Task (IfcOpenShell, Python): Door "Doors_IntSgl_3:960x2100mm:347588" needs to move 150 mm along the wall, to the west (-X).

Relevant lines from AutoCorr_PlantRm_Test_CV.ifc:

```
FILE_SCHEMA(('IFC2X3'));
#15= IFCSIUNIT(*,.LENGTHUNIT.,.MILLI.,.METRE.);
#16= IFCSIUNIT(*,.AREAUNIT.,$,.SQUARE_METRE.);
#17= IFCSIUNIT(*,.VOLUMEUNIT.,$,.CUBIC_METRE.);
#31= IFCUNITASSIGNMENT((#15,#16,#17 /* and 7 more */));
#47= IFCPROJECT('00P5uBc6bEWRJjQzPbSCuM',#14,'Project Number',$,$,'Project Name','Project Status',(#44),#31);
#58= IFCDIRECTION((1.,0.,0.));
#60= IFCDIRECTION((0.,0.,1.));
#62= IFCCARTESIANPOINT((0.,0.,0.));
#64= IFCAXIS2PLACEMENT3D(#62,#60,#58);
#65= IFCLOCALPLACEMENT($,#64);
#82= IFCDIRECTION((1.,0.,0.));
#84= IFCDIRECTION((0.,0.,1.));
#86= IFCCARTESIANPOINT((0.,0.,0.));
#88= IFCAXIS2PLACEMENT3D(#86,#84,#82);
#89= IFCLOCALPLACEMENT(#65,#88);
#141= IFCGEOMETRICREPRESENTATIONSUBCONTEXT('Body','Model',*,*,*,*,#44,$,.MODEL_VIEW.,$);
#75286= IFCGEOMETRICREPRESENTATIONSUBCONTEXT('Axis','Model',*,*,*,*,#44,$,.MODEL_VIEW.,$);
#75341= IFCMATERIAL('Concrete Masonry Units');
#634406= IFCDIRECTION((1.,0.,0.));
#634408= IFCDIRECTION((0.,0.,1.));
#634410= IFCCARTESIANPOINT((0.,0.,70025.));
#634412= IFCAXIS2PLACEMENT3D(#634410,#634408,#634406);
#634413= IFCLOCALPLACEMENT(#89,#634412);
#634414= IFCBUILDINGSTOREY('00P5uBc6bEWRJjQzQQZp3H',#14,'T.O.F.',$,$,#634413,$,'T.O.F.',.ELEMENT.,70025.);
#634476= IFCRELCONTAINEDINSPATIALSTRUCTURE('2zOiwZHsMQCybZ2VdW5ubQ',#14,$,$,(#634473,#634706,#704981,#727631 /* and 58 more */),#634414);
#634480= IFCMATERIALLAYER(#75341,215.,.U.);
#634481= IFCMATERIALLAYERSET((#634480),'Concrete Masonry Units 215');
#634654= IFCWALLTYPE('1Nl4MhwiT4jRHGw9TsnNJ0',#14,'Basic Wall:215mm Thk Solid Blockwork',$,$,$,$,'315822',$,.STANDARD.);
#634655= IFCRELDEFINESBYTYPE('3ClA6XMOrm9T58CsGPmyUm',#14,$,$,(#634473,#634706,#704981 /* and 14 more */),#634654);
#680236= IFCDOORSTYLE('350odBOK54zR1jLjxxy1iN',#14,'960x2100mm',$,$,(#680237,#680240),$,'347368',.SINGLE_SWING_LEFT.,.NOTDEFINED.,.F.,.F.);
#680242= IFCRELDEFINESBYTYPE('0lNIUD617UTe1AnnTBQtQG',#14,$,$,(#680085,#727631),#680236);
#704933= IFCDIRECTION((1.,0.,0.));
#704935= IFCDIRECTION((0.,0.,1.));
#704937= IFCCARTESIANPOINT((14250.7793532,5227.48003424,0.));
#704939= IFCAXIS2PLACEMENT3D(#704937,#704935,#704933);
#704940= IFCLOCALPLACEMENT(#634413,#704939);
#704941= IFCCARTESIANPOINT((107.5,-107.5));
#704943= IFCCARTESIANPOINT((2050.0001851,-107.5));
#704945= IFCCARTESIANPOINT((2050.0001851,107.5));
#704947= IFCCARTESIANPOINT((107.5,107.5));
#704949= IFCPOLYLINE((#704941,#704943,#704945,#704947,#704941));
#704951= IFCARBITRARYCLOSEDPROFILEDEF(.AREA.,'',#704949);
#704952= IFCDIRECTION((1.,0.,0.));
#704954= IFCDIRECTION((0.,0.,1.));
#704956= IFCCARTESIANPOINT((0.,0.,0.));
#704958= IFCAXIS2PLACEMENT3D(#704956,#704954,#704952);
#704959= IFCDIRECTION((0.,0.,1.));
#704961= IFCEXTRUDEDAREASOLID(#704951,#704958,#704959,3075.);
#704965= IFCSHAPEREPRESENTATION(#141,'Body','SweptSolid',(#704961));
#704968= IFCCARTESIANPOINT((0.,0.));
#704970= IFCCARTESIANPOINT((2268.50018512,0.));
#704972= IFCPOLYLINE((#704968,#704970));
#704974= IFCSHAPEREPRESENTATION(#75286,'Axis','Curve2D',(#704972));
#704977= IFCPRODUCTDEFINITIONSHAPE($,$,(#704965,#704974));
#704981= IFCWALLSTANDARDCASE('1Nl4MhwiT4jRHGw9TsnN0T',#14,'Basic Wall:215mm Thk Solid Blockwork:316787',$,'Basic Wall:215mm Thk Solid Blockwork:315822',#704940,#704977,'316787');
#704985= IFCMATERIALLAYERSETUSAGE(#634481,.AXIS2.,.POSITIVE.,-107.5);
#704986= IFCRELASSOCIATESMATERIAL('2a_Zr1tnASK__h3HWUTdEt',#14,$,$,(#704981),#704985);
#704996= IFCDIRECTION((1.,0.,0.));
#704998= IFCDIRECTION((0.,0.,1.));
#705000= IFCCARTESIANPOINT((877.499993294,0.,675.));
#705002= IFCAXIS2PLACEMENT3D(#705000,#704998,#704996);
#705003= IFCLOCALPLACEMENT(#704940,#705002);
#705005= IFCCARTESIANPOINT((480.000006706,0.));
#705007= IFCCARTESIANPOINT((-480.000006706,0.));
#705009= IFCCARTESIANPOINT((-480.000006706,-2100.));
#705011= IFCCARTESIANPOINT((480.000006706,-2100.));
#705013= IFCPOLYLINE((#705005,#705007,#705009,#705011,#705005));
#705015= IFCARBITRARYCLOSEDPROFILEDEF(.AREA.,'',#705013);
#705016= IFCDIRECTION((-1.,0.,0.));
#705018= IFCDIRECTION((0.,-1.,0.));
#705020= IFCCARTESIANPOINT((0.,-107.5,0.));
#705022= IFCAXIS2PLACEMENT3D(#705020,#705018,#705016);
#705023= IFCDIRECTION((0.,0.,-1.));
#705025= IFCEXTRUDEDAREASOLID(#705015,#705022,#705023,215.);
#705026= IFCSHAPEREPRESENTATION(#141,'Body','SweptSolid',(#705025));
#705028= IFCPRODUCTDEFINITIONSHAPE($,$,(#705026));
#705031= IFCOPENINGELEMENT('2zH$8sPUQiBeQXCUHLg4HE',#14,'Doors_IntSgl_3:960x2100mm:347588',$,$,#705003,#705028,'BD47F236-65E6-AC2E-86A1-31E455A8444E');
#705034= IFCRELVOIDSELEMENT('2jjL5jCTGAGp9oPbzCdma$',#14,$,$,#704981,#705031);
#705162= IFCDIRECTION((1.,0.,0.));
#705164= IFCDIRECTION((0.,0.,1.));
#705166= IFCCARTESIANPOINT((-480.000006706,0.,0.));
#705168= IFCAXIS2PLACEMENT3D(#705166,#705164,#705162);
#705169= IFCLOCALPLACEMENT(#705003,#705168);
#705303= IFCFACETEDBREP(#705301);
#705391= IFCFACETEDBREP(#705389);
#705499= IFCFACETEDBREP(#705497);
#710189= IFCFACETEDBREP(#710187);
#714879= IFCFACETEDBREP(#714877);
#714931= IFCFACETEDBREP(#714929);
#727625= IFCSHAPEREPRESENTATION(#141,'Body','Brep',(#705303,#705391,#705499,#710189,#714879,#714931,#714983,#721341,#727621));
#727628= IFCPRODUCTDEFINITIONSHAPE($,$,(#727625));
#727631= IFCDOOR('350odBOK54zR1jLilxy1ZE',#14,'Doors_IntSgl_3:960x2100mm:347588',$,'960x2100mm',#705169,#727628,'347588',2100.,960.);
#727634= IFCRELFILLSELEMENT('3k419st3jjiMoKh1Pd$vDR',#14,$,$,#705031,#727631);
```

```python
import ifcopenshell
import ifcopenshell.api.geometry
import ifcopenshell.util.placement

model = ifcopenshell.open("AutoCorr_PlantRm_Test_CV.ifc")

door = model.by_guid("350odBOK54zR1jLilxy1ZE")
opening = door.FillsVoids[0].RelatingOpeningElement
wall = opening.VoidsElements[0].RelatingBuildingElement

wall_matrix = ifcopenshell.util.placement.get_local_placement(wall.ObjectPlacement)
shift = wall_matrix[:3, 0] * -150.0
before = ifcopenshell.util.placement.get_local_placement(door.ObjectPlacement)[:3, 3].copy()

# The door is placed relative to its opening, so it follows when the opening moves.
matrix = ifcopenshell.util.placement.get_local_placement(opening.ObjectPlacement)
matrix[:3, 3] += shift
ifcopenshell.api.geometry.edit_object_placement(
    model, product=opening, matrix=matrix, is_si=False, should_transform_children=True
)

after = ifcopenshell.util.placement.get_local_placement(door.ObjectPlacement)[:3, 3]
print("door moved by", (after - before).round(3) + 0.0)

model.write("AutoCorr_PlantRm_Test_CV_edited.ifc")
```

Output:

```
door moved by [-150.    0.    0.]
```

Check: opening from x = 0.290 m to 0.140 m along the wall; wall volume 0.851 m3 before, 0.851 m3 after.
